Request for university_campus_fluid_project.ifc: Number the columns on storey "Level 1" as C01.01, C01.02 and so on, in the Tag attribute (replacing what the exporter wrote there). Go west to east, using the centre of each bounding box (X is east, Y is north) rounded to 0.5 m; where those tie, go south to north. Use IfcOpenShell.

First a look at what the model holds.

```python
import ifcopenshell
import ifcopenshell.util.element
import ifcopenshell.util.placement

model = ifcopenshell.open("university_campus_fluid_project.ifc")
print(model.schema)
storey = next(s for s in model.by_type("IfcBuildingStorey") if s.Name == "Level 1")
columns = [e for e in ifcopenshell.util.element.get_decomposition(storey) if e.is_a("IfcColumn")]
for e in sorted(columns, key=lambda e: e.id()):
    origin = ifcopenshell.util.placement.get_local_placement(e.ObjectPlacement)[:3, 3]
    print(e.id(), e.Tag, e.Name, origin.round(2) + 0.0, sep=" | ")
```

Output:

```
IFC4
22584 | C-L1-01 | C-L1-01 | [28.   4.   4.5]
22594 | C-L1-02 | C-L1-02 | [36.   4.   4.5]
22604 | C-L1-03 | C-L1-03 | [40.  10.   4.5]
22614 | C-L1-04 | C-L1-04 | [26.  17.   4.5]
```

```python
import ifcopenshell
import ifcopenshell.geom
import ifcopenshell.util.element
import ifcopenshell.util.shape

model = ifcopenshell.open("university_campus_fluid_project.ifc")
settings = ifcopenshell.geom.settings()
settings.set("use-world-coords", True)


def centre(element):
    shape = ifcopenshell.geom.create_shape(settings, element)
    return ifcopenshell.util.shape.get_bbox_centroid(shape.geometry)


storey = next(s for s in model.by_type("IfcBuildingStorey") if s.Name == "Level 1")
columns = [e for e in ifcopenshell.util.element.get_decomposition(storey) if e.is_a("IfcColumn")]

# Insertion points can sit at a corner or the storey origin, so sort by the geometry (in metres).
centres = {e: centre(e) for e in columns}
columns.sort(key=lambda e: (round(centres[e][0] / 0.5), centres[e][1]))

for i, e in enumerate(columns, start=1):
    number = f"C01.{i:02d}"
    e.Tag = number
    print(e.id(), number)

model.write("university_campus_fluid_project_v2.ifc")
```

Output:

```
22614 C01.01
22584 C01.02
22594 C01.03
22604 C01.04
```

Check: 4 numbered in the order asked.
